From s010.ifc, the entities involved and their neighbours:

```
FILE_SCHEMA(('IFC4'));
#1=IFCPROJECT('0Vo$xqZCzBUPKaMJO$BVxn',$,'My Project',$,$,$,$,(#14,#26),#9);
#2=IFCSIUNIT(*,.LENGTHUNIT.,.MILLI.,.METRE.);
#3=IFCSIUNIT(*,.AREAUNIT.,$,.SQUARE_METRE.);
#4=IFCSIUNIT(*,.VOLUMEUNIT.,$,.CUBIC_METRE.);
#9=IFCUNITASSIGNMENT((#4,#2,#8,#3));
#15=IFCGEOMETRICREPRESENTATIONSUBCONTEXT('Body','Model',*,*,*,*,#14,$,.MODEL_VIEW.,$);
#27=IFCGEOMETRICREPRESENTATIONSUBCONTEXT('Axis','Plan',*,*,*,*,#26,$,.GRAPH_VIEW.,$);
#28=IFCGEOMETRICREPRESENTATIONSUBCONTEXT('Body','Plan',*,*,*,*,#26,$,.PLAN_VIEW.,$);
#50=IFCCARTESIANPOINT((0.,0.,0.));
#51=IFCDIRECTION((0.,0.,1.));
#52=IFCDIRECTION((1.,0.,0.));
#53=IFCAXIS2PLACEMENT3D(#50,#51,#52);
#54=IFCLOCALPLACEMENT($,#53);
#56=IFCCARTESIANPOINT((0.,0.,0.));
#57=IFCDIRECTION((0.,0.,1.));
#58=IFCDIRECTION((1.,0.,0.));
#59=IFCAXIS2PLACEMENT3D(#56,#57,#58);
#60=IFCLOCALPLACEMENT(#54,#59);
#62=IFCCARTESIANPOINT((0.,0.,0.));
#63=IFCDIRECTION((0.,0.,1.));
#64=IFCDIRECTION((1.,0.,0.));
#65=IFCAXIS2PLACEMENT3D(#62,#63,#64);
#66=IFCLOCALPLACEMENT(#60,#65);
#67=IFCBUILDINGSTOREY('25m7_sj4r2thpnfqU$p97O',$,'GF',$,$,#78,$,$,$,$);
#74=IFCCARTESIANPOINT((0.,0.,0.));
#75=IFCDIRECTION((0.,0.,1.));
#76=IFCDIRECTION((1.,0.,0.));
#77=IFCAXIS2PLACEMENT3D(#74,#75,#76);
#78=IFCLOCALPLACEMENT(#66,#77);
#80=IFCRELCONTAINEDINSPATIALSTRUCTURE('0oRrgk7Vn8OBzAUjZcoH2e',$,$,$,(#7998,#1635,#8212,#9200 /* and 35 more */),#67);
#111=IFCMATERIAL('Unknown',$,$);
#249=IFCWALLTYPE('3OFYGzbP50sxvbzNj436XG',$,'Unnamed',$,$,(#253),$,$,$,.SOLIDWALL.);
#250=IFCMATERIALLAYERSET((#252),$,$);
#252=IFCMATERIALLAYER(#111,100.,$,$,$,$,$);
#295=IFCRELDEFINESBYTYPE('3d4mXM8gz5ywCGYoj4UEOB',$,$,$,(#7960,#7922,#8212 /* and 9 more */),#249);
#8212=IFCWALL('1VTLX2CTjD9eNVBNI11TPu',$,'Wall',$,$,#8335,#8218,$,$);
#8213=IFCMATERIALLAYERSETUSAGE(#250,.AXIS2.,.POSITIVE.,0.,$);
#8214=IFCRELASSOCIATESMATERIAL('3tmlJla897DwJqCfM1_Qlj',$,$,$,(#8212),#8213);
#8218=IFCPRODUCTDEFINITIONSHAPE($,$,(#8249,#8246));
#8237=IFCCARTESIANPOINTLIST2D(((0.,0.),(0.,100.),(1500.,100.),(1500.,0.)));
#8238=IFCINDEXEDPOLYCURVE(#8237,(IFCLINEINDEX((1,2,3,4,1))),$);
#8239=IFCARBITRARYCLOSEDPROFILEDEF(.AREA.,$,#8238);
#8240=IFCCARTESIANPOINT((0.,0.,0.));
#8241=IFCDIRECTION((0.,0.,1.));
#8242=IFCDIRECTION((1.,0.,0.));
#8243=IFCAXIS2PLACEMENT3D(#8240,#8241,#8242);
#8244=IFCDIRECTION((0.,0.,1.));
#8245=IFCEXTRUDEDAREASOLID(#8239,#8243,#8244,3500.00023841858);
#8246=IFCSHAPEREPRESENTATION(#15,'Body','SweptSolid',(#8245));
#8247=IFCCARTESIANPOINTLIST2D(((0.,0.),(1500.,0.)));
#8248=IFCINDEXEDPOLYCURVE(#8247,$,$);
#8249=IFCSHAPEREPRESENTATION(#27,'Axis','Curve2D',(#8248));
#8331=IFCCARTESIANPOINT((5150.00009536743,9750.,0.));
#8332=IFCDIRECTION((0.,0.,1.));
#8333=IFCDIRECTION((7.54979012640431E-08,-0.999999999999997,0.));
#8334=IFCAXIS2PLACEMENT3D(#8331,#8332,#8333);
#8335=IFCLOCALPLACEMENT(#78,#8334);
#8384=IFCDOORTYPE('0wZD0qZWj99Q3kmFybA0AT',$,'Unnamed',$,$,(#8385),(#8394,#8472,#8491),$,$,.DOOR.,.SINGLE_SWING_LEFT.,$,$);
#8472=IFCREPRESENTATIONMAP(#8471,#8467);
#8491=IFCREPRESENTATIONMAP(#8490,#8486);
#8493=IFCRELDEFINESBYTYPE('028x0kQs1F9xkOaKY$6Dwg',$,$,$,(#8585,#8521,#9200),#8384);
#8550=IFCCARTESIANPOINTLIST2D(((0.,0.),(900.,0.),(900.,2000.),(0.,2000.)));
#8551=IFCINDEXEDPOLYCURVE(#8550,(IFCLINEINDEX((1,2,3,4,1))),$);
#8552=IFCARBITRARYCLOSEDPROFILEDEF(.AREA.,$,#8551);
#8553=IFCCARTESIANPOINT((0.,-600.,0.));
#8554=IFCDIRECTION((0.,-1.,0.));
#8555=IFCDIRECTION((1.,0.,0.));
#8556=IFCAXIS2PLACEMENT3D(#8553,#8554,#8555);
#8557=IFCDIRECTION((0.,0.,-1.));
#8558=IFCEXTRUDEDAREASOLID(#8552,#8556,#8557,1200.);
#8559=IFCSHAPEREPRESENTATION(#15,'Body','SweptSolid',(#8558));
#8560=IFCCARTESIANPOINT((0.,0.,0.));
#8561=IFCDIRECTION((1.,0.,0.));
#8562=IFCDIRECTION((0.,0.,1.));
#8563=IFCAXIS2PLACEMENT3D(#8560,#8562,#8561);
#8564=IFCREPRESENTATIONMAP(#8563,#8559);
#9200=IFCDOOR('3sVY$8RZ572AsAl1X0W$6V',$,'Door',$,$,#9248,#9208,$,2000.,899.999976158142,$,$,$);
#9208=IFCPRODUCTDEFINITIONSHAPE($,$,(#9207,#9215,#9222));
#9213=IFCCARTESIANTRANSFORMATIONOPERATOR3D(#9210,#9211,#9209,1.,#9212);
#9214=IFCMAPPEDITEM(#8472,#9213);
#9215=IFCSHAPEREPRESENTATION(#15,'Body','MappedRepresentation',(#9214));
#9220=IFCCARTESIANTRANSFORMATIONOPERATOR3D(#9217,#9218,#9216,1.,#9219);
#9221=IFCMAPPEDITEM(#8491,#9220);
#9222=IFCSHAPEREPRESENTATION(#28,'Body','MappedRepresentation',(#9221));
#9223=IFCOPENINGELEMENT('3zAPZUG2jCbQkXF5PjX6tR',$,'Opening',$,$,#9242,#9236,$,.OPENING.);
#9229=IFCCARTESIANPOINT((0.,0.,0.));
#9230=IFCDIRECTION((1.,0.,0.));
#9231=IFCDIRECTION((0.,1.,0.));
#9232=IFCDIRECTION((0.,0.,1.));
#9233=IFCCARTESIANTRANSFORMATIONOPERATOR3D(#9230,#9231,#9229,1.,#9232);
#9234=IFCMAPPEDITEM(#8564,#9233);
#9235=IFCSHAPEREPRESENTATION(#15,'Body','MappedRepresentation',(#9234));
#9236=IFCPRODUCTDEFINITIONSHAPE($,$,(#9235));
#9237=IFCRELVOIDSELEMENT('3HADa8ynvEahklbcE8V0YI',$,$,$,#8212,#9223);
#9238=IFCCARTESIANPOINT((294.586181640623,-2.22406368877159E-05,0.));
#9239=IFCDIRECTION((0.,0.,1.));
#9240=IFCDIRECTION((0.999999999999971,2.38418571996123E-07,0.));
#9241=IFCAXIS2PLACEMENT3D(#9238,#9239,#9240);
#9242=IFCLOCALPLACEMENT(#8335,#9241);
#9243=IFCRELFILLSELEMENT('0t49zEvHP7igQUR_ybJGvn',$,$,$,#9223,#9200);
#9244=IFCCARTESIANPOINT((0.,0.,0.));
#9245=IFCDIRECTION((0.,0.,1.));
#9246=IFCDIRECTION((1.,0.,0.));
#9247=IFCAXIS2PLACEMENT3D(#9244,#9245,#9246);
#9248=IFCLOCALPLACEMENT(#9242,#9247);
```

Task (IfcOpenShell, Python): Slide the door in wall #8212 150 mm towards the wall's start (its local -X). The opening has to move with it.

```python
import ifcopenshell
import ifcopenshell.api.geometry
import ifcopenshell.util.placement
import ifcopenshell.util.unit

model = ifcopenshell.open("s010.ifc")
unit_scale = ifcopenshell.util.unit.calculate_unit_scale(model)

door = model.by_guid("3sVY$8RZ572AsAl1X0W$6V")
opening = door.FillsVoids[0].RelatingOpeningElement
wall = opening.VoidsElements[0].RelatingBuildingElement

wall_matrix = ifcopenshell.util.placement.get_local_placement(wall.ObjectPlacement)
shift = wall_matrix[:3, 0] * -0.15 / unit_scale
before = ifcopenshell.util.placement.get_local_placement(door.ObjectPlacement)[:3, 3].copy()

# The door is placed relative to its opening, so it follows when the opening moves.
matrix = ifcopenshell.util.placement.get_local_placement(opening.ObjectPlacement)
matrix[:3, 3] += shift
ifcopenshell.api.geometry.edit_object_placement(
    model, product=opening, matrix=matrix, is_si=False, should_transform_children=True
)

after = ifcopenshell.util.placement.get_local_placement(door.ObjectPlacement)[:3, 3]
print("door moved by", (after - before).round(3) + 0.0)

model.write("s010_updated.ifc")
```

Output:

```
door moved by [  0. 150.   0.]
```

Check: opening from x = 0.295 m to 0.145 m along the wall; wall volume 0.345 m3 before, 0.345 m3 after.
